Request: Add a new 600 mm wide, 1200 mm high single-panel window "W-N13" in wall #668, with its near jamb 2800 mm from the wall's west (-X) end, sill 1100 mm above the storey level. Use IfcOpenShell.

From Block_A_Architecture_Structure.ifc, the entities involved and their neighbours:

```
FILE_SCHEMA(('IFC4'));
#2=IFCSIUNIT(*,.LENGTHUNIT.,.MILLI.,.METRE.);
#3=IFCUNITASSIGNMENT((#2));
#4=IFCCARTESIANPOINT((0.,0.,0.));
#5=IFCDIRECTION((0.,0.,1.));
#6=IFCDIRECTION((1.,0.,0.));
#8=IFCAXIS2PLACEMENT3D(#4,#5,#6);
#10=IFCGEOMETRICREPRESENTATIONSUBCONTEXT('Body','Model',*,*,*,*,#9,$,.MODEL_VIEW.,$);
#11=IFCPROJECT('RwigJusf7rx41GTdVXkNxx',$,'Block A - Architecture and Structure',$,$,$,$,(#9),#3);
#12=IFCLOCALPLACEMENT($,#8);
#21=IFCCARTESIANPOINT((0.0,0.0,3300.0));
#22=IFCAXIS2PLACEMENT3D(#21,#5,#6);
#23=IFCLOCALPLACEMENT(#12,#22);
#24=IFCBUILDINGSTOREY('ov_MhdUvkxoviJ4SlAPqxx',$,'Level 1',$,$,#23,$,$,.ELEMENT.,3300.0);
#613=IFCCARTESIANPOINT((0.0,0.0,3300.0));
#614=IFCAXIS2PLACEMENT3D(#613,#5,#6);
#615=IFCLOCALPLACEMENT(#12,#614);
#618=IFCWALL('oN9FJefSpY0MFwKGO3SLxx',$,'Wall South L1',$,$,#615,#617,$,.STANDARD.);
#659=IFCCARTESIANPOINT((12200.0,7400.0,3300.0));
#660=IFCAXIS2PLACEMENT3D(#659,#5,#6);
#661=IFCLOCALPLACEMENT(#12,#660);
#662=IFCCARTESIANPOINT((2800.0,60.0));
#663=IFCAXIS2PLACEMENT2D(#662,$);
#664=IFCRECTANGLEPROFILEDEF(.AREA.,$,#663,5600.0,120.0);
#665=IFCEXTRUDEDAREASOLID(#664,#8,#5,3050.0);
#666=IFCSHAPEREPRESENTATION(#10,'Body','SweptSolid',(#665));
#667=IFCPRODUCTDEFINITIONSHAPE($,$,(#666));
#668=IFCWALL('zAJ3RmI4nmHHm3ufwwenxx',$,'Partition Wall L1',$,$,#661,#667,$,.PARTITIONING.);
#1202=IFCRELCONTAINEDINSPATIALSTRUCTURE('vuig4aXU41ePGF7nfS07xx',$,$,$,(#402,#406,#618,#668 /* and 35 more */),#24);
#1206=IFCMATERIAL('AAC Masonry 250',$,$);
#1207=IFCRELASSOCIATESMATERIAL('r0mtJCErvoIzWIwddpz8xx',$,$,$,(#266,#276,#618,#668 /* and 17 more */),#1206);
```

```python
import numpy as np
import ifcopenshell
import ifcopenshell.api.feature
import ifcopenshell.api.geometry
import ifcopenshell.api.root
import ifcopenshell.api.spatial
import ifcopenshell.geom
import ifcopenshell.util.element
import ifcopenshell.util.placement
import ifcopenshell.util.representation
import ifcopenshell.util.shape
import ifcopenshell.util.unit

model = ifcopenshell.open("Block_A_Architecture_Structure.ifc")
unit_scale = ifcopenshell.util.unit.calculate_unit_scale(model)
settings = ifcopenshell.geom.settings()


def volume(element):
    """Net volume in cubic metres, openings subtracted."""
    shape = ifcopenshell.geom.create_shape(settings, element)
    return ifcopenshell.util.shape.get_volume(shape.geometry)


wall = model.by_guid("zAJ3RmI4nmHHm3ufwwenxx")
storey = ifcopenshell.util.element.get_container(wall, ifc_class="IfcBuildingStorey")
context = ifcopenshell.util.representation.get_context(model, "Model", "Body", "MODEL_VIEW")
before = volume(wall)

width, height, from_end, sill = 0.6, 1.2, 2.8, 1.1  # metres

# The wall runs along its own X axis, and the end named is its -X end.
wall_shape = ifcopenshell.geom.create_shape(settings, wall)
x, y, z = ifcopenshell.util.shape.get_vertices(wall_shape.geometry).T
start = x.min() + from_end
face, thickness = float(y.min()), float(y.max() - y.min())
wall_matrix = ifcopenshell.util.placement.get_local_placement(wall.ObjectPlacement)
level = ifcopenshell.util.placement.get_local_placement(storey.ObjectPlacement)[2, 3]


def in_wall(x, y):
    """Placement at x, y metres in the wall's axes, at sill height."""
    matrix = wall_matrix.copy()
    matrix[:, 3] = wall_matrix @ np.array([x / unit_scale, y / unit_scale, 0.0, 1.0])
    matrix[2, 3] = level + sill / unit_scale
    return matrix


# Opening: a box that overshoots both wall faces by 50 mm.
opening = ifcopenshell.api.root.create_entity(model, ifc_class="IfcOpeningElement", predefined_type="OPENING")
box = ifcopenshell.api.geometry.add_wall_representation(
    model, context=context, length=width, height=height, thickness=thickness + 0.1
)
ifcopenshell.api.geometry.assign_representation(model, product=opening, representation=box)
ifcopenshell.api.geometry.edit_object_placement(model, product=opening, matrix=in_wall(start, face - 0.05), is_si=False)
ifcopenshell.api.feature.add_feature(model, feature=opening, element=wall)

window = ifcopenshell.api.root.create_entity(model, ifc_class="IfcWindow", name="W-N13", predefined_type="WINDOW")
window.OverallWidth, window.OverallHeight = width / unit_scale, height / unit_scale
window.PartitioningType = "SINGLE_PANEL"
body = ifcopenshell.api.geometry.add_window_representation(
    model,
    context=context,
    overall_width=window.OverallWidth,
    overall_height=window.OverallHeight,
    partition_type="SINGLE_PANEL",
)
ifcopenshell.api.geometry.assign_representation(model, product=window, representation=body)
ifcopenshell.api.spatial.assign_container(model, products=[window], relating_structure=storey)
ifcopenshell.api.feature.add_filling(model, opening=opening, element=window)

# Centre the window in the wall's thickness.
ifcopenshell.api.geometry.edit_object_placement(model, product=window, matrix=in_wall(start, face), is_si=False)
window_shape = ifcopenshell.geom.create_shape(settings, window)
depth = ifcopenshell.util.shape.get_vertices(window_shape.geometry)[:, 1]
offset = face + thickness / 2 - (depth.min() + depth.max()) / 2
ifcopenshell.api.geometry.edit_object_placement(model, product=window, matrix=in_wall(start, offset), is_si=False)

after = volume(wall)

print(f"wall volume {before:.3f} -> {after:.3f} m3")

model.write("Block_A_Architecture_Structure_rev.ifc")
```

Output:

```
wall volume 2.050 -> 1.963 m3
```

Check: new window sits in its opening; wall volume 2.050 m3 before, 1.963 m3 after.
